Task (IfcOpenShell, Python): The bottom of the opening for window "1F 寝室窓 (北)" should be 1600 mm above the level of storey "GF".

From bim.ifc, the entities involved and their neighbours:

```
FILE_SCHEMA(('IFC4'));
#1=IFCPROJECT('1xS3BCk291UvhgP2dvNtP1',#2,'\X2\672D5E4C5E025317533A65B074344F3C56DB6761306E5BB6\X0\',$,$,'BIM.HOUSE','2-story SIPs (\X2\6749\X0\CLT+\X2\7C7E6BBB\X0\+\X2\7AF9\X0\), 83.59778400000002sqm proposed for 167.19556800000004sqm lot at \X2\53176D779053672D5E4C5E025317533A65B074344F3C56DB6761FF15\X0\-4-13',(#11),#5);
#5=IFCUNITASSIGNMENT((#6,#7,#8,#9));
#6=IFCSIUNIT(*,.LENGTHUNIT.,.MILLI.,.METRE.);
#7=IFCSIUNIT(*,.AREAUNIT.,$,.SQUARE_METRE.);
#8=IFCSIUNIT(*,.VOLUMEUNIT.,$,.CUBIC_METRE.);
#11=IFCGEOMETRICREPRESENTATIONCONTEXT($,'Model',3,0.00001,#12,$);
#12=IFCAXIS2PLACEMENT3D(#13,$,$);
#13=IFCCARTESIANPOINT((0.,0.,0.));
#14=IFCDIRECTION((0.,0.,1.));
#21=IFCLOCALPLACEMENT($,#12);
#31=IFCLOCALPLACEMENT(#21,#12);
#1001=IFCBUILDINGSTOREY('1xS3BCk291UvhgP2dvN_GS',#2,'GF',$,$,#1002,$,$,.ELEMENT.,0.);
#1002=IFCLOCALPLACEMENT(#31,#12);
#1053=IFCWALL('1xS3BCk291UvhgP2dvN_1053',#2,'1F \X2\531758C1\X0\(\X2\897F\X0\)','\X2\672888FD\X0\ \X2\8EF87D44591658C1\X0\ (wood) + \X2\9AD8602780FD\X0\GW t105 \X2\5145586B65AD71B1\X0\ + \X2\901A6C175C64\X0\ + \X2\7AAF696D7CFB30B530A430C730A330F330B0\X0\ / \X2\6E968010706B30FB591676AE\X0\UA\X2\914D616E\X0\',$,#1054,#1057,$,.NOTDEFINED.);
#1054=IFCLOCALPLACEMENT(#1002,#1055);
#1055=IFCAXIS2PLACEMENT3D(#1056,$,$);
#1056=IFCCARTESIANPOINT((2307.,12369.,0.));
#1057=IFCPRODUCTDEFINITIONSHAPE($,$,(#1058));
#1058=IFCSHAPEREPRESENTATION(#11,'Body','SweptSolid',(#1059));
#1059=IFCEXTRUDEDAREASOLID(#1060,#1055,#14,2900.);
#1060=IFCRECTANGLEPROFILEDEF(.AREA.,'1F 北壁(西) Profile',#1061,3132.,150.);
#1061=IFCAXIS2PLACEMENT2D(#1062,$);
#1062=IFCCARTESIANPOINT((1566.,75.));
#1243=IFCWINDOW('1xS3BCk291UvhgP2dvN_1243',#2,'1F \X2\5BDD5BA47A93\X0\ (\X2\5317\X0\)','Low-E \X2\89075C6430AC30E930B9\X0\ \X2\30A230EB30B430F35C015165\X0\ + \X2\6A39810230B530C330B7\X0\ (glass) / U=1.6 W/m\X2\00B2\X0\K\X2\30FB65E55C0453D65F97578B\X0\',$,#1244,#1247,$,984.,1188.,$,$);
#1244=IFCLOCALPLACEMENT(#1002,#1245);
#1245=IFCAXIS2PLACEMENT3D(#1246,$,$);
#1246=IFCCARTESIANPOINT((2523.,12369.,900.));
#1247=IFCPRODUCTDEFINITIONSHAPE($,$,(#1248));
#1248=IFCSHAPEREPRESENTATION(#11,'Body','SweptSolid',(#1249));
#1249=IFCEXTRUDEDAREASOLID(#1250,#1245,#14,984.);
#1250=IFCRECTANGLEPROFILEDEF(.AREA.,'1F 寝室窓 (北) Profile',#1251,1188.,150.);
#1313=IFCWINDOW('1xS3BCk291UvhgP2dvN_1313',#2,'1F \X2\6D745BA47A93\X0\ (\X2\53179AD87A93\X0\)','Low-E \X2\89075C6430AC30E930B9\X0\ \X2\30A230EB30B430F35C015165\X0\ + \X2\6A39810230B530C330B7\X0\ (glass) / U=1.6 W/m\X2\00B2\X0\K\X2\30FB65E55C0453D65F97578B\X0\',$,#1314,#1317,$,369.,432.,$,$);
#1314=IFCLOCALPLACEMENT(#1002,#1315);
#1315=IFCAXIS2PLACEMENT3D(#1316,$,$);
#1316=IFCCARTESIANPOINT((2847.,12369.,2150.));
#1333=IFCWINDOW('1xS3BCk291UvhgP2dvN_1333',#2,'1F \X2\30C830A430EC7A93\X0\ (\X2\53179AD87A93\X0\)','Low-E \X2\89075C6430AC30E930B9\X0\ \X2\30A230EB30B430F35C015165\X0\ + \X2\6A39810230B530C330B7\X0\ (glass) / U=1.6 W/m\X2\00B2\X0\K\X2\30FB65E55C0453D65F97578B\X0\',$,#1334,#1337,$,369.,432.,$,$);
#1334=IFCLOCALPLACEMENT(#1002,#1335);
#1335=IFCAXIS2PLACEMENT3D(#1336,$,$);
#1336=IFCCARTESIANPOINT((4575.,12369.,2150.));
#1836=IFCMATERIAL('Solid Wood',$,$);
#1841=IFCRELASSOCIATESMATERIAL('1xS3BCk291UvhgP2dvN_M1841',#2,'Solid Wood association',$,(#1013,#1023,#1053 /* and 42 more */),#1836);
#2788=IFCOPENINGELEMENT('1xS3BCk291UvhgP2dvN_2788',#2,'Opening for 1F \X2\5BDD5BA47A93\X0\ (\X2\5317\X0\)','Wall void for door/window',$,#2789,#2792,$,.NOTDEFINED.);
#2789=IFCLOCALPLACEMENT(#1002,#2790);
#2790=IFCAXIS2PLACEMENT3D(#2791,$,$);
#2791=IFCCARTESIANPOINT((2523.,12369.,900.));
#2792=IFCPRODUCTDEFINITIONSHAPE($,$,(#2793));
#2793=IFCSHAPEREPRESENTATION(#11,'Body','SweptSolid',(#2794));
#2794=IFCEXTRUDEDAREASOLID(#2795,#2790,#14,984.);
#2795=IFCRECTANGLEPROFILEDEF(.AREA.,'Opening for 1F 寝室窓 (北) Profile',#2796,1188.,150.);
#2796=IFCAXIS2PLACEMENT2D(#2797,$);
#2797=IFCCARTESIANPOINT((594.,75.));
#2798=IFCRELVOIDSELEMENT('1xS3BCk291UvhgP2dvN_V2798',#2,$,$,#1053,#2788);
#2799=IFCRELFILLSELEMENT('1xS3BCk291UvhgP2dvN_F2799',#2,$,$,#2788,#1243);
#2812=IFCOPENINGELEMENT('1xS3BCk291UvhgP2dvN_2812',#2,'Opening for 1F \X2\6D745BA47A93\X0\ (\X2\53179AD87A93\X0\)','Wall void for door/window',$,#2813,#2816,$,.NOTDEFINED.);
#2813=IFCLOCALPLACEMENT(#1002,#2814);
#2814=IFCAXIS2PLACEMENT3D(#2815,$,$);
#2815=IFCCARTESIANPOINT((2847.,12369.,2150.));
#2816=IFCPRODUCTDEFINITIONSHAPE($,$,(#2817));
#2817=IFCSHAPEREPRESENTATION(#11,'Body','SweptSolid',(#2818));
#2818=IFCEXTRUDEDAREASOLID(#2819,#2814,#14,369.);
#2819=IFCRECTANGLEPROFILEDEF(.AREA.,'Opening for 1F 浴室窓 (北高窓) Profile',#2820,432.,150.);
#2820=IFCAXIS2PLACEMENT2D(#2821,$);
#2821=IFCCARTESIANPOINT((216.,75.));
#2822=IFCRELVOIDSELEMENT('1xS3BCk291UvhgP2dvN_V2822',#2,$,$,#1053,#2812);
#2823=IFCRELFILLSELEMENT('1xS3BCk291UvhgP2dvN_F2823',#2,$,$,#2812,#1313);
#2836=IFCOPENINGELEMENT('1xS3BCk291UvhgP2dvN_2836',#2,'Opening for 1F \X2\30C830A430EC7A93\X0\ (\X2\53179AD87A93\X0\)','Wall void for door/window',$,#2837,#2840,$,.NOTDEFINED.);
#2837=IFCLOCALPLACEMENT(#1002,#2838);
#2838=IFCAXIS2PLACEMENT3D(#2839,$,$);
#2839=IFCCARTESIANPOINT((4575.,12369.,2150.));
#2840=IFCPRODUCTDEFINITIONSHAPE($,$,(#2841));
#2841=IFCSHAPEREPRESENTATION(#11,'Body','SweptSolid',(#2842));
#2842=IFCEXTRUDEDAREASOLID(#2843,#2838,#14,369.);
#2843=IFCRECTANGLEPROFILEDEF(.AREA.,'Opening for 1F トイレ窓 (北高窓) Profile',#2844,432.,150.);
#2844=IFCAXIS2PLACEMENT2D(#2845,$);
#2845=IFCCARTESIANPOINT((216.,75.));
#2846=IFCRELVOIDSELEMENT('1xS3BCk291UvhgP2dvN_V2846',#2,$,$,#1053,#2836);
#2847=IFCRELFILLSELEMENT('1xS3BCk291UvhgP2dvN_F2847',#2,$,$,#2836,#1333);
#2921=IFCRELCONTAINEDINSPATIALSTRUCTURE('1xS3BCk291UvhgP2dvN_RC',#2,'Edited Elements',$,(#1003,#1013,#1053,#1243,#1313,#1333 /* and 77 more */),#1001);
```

```python
import numpy as np
import ifcopenshell
import ifcopenshell.api.geometry
import ifcopenshell.geom
import ifcopenshell.util.element
import ifcopenshell.util.placement
import ifcopenshell.util.shape
import ifcopenshell.util.unit

model = ifcopenshell.open("bim.ifc")
unit_scale = ifcopenshell.util.unit.calculate_unit_scale(model)

window = model.by_guid("1xS3BCk291UvhgP2dvN_1243")
opening = window.FillsVoids[0].RelatingOpeningElement
storey = ifcopenshell.util.element.get_container(window, ifc_class="IfcBuildingStorey")
level = ifcopenshell.util.placement.get_local_placement(storey.ObjectPlacement)[2, 3]

# The opening's origin need not be at the sill, so measure its lowest point.
shape = ifcopenshell.geom.create_shape(ifcopenshell.geom.settings(), opening)
bottom = ifcopenshell.util.shape.get_shape_bottom_elevation(shape, shape.geometry) / unit_scale
dz = level + 1600.0 - bottom

shift = np.array([0.0, 0.0, dz])
# The window is not placed relative to its opening, so move both.
for product in (opening, window):
    matrix = ifcopenshell.util.placement.get_local_placement(product.ObjectPlacement)
    matrix[:3, 3] += shift
    ifcopenshell.api.geometry.edit_object_placement(model, product=product, matrix=matrix, is_si=False)

print(f"moved by {dz * unit_scale:+.3f} m")

model.write("bim_edited.ifc")
```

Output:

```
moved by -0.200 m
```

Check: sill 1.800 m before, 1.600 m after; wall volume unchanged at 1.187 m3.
